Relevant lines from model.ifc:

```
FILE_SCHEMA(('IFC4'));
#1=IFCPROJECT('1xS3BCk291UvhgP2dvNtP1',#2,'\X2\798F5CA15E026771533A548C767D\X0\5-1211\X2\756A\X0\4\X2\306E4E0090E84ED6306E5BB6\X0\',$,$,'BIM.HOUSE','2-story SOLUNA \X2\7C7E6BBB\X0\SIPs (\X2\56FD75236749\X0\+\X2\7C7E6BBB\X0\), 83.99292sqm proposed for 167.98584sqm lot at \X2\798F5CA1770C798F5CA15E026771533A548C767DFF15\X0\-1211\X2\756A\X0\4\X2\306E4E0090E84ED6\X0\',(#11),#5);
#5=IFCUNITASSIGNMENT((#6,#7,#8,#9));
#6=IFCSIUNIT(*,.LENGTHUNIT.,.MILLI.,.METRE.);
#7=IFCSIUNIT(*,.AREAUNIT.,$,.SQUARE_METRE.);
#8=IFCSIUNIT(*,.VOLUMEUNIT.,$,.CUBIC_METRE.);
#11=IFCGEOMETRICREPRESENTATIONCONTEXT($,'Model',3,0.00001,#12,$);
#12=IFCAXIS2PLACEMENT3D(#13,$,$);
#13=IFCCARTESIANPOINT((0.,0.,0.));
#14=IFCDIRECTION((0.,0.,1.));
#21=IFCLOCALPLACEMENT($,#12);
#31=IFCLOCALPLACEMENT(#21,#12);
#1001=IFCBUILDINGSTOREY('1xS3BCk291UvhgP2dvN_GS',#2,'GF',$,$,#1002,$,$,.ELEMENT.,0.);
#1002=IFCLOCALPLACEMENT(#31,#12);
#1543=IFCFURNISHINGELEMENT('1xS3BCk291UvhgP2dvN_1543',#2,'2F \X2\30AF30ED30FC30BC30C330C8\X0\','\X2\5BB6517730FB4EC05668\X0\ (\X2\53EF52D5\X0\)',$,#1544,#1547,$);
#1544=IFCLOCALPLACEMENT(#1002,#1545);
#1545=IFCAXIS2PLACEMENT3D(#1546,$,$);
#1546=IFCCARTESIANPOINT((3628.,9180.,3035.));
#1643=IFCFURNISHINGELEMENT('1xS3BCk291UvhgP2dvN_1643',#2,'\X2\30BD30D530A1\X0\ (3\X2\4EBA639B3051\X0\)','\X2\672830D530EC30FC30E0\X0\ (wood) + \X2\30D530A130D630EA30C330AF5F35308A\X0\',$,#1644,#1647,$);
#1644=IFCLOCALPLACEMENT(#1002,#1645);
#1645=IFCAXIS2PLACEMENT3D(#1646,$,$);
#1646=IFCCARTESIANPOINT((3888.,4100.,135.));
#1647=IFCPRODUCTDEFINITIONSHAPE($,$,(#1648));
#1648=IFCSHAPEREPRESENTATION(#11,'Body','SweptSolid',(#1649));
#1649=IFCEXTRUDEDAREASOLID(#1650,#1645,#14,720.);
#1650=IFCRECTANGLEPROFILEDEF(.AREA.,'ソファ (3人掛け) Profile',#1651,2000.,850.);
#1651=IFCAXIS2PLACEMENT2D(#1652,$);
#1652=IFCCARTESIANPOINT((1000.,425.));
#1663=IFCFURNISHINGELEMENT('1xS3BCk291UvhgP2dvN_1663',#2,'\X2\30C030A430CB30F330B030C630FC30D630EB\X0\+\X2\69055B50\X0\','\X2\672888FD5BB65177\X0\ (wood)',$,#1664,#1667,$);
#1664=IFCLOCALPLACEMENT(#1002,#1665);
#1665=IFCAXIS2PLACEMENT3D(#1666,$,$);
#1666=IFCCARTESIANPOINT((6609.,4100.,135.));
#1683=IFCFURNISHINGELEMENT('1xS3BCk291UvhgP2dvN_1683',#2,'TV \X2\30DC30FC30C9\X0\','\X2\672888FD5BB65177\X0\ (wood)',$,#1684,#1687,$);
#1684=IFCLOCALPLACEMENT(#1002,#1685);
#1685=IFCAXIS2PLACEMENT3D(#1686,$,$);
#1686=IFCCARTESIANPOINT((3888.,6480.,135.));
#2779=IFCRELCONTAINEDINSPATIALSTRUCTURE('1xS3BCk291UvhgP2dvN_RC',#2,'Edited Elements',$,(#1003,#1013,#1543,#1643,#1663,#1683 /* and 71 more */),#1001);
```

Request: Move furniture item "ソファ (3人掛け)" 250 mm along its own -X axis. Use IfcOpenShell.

```python
import ifcopenshell
import ifcopenshell.api.geometry
import ifcopenshell.util.placement

model = ifcopenshell.open("model.ifc")

item = model.by_guid("1xS3BCk291UvhgP2dvN_1643")
matrix = ifcopenshell.util.placement.get_local_placement(item.ObjectPlacement)
matrix[:3, 3] -= matrix[:3, 0] * 250.0
ifcopenshell.api.geometry.edit_object_placement(model, product=item, matrix=matrix, is_si=False)

print(ifcopenshell.util.placement.get_local_placement(item.ObjectPlacement).round(3) + 0.0)

model.write("model_rev.ifc")
```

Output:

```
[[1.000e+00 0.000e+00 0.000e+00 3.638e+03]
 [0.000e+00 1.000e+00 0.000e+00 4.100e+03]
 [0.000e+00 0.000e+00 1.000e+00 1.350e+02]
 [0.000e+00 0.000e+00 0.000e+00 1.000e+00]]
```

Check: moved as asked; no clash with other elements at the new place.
